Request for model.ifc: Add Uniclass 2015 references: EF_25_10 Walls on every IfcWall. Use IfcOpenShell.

First a look at what the model holds.

```python
import ifcopenshell

model = ifcopenshell.open("model.ifc")
print(model.schema)
print("classifications:", [c.Name for c in model.by_type("IfcClassification")])
for ifc_class in ("IfcDoor", "IfcRoof", "IfcStair", "IfcWall", "IfcWindow"):
    print(ifc_class, len(model.by_type(ifc_class)))
```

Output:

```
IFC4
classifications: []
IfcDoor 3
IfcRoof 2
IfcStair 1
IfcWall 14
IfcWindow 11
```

```python
import ifcopenshell
import ifcopenshell.api.classification

model = ifcopenshell.open("model.ifc")

system = ifcopenshell.api.classification.add_classification(model, classification="Uniclass 2015")

codes = {
    "IfcWall": ("EF_25_10", "Walls"),
}
for ifc_class, (code, name) in codes.items():
    products = model.by_type(ifc_class)
    ifcopenshell.api.classification.add_reference(
        model, products=products, classification=system, identification=code, name=name
    )
    print(code, len(products))

model.write("model_rev.ifc")
```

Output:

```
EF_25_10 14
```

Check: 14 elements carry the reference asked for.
